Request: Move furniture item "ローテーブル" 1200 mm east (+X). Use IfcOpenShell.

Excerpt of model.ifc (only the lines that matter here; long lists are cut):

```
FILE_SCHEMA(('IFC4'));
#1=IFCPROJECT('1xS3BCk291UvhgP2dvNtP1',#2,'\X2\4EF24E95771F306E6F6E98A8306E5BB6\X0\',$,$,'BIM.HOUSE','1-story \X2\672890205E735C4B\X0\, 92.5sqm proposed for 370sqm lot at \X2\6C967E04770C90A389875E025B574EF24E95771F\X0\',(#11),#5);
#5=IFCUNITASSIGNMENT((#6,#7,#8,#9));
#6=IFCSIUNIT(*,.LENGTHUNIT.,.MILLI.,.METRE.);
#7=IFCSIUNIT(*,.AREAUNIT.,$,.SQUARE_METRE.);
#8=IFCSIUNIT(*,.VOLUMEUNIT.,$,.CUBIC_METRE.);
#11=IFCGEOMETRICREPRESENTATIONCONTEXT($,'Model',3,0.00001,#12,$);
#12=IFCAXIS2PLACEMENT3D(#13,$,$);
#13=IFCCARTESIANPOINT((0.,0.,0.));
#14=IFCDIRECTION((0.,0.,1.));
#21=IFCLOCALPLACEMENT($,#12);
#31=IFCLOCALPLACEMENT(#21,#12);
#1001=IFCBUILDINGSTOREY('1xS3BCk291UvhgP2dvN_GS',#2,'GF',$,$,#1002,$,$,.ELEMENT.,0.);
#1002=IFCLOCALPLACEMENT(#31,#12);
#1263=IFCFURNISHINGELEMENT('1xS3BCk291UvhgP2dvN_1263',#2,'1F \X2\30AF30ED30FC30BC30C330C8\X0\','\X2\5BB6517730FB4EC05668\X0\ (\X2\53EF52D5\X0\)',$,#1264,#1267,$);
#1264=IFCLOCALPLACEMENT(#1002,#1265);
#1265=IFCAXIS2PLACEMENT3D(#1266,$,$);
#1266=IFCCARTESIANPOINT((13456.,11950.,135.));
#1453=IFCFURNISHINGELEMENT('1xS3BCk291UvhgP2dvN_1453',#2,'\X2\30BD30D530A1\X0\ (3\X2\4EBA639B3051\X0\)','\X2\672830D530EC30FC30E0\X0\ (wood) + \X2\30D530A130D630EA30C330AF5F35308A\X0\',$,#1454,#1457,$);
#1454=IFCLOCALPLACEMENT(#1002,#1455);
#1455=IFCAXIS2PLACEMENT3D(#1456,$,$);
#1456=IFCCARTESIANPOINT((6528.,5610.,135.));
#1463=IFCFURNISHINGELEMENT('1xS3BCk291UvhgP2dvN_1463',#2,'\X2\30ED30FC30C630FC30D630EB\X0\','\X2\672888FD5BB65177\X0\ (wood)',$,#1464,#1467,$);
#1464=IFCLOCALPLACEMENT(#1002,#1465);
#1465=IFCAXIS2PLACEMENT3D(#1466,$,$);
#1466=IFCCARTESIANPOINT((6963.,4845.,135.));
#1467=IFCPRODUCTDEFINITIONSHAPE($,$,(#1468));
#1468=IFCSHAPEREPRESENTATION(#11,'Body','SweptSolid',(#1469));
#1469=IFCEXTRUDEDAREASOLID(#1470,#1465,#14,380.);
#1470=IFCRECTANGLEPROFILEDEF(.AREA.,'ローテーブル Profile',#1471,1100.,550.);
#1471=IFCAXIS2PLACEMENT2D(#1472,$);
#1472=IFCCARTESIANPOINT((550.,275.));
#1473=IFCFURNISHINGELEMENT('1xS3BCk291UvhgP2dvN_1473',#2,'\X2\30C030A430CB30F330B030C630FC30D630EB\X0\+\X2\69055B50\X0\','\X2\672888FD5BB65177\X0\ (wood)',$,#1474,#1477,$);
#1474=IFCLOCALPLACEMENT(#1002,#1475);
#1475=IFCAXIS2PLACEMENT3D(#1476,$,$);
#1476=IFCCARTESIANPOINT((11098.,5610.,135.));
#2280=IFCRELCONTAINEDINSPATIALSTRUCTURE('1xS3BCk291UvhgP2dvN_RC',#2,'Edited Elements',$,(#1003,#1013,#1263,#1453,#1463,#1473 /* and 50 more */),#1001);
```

```python
import ifcopenshell
import ifcopenshell.api.geometry
import ifcopenshell.util.placement

model = ifcopenshell.open("model.ifc")

item = model.by_guid("1xS3BCk291UvhgP2dvN_1463")
matrix = ifcopenshell.util.placement.get_local_placement(item.ObjectPlacement)
matrix[0, 3] += 1200.0
ifcopenshell.api.geometry.edit_object_placement(model, product=item, matrix=matrix, is_si=False)

print(ifcopenshell.util.placement.get_local_placement(item.ObjectPlacement).round(3) + 0.0)

model.write("model_edited.ifc")
```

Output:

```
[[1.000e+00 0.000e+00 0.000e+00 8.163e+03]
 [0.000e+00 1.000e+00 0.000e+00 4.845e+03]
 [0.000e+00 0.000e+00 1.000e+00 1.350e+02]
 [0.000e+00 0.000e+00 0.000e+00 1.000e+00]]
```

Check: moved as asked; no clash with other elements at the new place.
